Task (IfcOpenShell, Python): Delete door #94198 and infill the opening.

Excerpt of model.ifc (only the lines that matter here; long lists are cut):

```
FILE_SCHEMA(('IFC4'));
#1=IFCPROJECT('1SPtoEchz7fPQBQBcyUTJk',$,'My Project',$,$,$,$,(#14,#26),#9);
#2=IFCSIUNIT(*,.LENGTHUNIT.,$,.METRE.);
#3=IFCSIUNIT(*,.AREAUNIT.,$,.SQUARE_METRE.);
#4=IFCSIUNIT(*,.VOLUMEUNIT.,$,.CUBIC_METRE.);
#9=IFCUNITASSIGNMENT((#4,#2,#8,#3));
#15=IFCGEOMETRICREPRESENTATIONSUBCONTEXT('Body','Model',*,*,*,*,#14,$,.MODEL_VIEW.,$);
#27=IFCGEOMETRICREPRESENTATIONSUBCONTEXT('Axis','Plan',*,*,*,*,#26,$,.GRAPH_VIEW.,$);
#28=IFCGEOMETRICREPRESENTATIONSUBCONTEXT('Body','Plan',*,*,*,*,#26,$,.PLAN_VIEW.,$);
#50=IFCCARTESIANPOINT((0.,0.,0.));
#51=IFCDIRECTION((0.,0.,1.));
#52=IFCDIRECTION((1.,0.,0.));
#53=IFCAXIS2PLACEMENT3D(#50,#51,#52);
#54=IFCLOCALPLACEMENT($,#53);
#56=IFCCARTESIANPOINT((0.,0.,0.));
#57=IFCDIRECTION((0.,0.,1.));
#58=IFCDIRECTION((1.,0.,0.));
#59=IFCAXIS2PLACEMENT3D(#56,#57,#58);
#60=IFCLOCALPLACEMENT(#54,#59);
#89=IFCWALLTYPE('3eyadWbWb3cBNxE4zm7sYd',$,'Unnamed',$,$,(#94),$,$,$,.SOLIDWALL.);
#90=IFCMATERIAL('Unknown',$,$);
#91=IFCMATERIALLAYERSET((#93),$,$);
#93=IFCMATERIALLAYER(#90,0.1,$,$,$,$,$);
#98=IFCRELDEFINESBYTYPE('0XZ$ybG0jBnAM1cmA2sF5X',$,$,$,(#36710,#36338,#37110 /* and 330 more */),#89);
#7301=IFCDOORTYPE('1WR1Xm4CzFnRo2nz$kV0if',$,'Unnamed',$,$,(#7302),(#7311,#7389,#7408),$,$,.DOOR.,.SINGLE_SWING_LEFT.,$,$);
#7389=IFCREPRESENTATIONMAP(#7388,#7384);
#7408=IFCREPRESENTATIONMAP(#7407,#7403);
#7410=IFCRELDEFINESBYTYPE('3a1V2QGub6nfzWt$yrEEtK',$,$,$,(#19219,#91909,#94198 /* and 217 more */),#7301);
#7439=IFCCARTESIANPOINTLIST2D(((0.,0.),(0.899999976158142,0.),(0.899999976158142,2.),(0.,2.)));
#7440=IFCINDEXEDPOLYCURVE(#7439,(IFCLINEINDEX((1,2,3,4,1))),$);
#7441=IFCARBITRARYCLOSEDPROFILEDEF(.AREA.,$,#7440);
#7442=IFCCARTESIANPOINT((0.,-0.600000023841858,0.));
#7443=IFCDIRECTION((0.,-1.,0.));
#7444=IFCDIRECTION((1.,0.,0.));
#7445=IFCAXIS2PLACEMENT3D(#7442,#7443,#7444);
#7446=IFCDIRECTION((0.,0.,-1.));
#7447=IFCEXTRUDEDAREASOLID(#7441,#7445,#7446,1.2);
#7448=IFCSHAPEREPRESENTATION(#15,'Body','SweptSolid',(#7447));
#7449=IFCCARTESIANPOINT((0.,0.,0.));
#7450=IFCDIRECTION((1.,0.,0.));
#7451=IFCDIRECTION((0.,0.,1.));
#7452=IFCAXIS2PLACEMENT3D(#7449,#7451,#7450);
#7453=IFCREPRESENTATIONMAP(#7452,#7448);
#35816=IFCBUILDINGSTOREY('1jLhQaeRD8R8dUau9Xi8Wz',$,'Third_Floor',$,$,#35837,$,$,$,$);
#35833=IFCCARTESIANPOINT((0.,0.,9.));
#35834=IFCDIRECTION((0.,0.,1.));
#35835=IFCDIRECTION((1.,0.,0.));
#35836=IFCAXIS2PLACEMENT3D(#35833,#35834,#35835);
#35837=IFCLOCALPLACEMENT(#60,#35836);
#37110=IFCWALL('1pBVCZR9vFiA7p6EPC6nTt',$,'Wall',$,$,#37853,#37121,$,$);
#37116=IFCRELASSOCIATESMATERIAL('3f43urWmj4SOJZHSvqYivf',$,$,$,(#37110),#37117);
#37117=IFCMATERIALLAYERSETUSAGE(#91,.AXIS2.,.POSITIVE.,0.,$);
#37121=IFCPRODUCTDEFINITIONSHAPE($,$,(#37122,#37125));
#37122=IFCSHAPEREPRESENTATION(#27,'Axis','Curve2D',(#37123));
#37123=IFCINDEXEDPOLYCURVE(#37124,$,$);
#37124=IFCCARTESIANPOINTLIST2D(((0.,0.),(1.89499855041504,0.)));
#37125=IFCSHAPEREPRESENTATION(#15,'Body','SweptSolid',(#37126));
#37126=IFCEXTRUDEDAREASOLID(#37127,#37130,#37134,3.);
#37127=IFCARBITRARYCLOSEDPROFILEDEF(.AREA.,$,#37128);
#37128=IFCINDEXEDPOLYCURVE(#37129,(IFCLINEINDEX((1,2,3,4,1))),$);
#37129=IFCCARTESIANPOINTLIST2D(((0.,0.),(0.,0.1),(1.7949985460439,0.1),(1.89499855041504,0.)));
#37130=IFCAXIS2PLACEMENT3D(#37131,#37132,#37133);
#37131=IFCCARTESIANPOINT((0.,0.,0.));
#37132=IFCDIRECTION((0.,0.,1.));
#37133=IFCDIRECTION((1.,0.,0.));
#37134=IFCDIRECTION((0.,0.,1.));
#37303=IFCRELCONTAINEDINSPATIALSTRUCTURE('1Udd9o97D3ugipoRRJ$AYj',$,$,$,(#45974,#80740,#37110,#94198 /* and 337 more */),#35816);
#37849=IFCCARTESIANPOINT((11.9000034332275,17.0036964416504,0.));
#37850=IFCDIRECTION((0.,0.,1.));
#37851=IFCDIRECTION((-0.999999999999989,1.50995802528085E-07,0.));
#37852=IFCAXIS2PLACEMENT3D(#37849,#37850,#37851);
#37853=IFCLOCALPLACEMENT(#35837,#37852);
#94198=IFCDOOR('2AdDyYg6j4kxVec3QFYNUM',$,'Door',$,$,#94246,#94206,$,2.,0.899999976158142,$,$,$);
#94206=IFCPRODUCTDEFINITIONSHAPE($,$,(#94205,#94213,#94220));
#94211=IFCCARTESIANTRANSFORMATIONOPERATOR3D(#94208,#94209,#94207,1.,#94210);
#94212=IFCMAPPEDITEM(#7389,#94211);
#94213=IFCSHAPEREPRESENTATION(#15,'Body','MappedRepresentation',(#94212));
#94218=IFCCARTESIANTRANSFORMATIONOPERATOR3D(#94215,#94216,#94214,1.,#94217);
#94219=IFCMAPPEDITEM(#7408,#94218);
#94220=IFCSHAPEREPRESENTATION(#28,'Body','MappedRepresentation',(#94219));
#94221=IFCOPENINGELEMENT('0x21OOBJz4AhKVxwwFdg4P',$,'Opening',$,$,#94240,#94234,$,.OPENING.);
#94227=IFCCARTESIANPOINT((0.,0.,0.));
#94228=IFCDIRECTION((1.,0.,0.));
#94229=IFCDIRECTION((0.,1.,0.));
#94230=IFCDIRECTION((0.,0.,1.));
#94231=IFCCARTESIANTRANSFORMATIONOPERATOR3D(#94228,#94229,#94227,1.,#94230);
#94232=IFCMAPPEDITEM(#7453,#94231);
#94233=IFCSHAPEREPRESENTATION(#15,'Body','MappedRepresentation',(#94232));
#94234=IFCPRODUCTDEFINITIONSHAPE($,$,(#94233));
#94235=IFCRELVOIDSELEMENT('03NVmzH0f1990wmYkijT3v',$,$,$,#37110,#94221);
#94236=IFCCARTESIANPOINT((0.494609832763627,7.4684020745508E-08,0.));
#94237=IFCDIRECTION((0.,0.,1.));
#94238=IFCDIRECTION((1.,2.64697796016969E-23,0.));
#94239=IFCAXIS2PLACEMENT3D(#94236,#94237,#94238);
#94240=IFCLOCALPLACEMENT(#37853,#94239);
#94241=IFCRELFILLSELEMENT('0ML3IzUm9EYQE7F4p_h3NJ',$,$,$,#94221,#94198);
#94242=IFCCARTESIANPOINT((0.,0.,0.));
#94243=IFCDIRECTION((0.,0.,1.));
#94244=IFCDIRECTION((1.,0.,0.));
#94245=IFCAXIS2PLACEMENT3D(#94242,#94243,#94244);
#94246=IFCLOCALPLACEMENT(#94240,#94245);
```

```python
import ifcopenshell
import ifcopenshell.api.feature
import ifcopenshell.api.root
import ifcopenshell.geom
import ifcopenshell.util.shape

model = ifcopenshell.open("model.ifc")
settings = ifcopenshell.geom.settings()


def volume(element):
    """Net volume in cubic metres, openings subtracted."""
    shape = ifcopenshell.geom.create_shape(settings, element)
    return ifcopenshell.util.shape.get_volume(shape.geometry)


door = model.by_id(94198)
opening = door.FillsVoids[0].RelatingOpeningElement
wall = opening.VoidsElements[0].RelatingBuildingElement
before = volume(wall)

ifcopenshell.api.root.remove_product(model, product=door)
ifcopenshell.api.feature.remove_feature(model, feature=opening)

after = volume(wall)

print(f"wall volume {before:.3f} -> {after:.3f} m3")

model.write("model_v2.ifc")
```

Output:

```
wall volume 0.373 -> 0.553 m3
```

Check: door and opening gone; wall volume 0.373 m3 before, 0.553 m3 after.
